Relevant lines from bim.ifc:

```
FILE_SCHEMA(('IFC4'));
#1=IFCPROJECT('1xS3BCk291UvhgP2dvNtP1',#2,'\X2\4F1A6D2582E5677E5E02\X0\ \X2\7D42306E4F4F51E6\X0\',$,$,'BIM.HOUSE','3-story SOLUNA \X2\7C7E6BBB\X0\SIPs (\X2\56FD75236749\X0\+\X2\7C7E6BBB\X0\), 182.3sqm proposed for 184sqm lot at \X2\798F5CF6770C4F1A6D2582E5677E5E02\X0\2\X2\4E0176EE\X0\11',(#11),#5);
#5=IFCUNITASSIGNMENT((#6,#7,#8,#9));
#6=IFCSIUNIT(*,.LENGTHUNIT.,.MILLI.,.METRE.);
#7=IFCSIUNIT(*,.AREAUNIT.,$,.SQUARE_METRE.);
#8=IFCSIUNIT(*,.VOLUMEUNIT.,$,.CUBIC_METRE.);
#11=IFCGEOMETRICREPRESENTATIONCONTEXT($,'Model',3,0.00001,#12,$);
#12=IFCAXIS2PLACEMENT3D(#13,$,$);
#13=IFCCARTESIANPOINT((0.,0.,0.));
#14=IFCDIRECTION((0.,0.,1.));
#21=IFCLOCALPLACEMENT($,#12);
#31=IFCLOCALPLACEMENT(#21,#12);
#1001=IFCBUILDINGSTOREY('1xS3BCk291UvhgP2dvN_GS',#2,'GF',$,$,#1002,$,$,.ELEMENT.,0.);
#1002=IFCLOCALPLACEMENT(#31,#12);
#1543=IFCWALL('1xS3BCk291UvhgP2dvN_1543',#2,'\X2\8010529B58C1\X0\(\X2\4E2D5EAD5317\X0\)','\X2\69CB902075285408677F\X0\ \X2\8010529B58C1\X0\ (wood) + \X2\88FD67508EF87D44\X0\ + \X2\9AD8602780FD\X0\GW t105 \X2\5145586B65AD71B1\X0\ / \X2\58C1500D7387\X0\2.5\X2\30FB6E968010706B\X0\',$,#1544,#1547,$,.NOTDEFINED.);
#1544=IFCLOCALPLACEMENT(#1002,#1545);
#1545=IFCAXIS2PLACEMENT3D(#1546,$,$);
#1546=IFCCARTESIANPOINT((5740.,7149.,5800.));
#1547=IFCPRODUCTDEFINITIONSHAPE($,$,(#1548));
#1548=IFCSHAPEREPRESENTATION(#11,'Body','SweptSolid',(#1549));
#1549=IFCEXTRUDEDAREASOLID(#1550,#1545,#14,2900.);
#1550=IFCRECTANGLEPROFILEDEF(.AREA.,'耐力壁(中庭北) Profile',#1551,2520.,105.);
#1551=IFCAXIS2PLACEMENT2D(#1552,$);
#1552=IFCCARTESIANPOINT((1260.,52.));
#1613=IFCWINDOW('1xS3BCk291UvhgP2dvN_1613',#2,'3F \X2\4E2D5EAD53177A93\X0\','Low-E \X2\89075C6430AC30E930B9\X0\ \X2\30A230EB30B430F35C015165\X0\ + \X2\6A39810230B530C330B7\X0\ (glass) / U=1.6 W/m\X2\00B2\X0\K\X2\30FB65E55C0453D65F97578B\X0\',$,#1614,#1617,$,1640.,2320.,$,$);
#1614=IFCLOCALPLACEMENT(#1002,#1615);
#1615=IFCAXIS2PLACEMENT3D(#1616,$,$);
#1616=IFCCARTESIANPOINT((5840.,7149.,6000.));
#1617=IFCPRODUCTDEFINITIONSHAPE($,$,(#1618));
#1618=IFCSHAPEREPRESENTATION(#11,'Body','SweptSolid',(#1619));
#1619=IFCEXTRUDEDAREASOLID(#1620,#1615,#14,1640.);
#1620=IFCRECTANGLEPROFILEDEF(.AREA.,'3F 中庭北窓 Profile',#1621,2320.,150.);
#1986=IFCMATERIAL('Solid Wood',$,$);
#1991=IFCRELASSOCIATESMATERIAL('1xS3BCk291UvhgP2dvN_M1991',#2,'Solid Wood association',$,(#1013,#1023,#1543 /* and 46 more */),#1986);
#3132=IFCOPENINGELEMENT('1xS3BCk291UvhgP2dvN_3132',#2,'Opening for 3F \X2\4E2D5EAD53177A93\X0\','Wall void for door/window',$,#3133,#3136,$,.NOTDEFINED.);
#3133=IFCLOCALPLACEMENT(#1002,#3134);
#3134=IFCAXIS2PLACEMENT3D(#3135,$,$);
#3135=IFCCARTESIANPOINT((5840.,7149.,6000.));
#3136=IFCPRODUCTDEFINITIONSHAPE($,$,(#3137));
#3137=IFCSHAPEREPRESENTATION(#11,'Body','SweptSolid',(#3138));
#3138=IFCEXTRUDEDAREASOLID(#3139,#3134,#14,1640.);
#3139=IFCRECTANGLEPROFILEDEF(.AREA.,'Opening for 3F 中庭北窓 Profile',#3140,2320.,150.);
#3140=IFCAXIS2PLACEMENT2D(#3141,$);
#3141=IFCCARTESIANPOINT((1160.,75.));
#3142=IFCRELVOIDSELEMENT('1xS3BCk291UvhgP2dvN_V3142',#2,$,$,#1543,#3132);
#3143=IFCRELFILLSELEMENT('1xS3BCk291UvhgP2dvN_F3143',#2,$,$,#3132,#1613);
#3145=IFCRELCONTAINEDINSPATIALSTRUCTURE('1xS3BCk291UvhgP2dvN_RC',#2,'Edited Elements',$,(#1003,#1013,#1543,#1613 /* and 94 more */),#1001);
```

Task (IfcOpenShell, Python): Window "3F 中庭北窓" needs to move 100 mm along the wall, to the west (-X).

```python
import ifcopenshell
import ifcopenshell.api.geometry
import ifcopenshell.util.placement

model = ifcopenshell.open("bim.ifc")

window = model.by_guid("1xS3BCk291UvhgP2dvN_1613")
opening = window.FillsVoids[0].RelatingOpeningElement
wall = opening.VoidsElements[0].RelatingBuildingElement

wall_matrix = ifcopenshell.util.placement.get_local_placement(wall.ObjectPlacement)
shift = wall_matrix[:3, 0] * -100.0
before = ifcopenshell.util.placement.get_local_placement(window.ObjectPlacement)[:3, 3].copy()

# The window is not placed relative to its opening, so move both.
for product in (opening, window):
    matrix = ifcopenshell.util.placement.get_local_placement(product.ObjectPlacement)
    matrix[:3, 3] += shift
    ifcopenshell.api.geometry.edit_object_placement(model, product=product, matrix=matrix, is_si=False)

after = ifcopenshell.util.placement.get_local_placement(window.ObjectPlacement)[:3, 3]
print("window moved by", (after - before).round(3) + 0.0)

model.write("bim_v2.ifc")
```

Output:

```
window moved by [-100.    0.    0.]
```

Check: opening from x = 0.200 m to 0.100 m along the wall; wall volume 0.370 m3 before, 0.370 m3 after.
